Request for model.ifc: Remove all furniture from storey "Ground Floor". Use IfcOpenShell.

First a look at what the model holds.

```python
import ifcopenshell
import ifcopenshell.util.element

model = ifcopenshell.open("model.ifc")
print(model.schema)
storey = next(s for s in model.by_type("IfcBuildingStorey") if s.Name == "Ground Floor")
furniture = [e for e in ifcopenshell.util.element.get_decomposition(storey) if e.is_a("IfcFurnishingElement")]
seen = {}
for e in furniture:
    element_type = ifcopenshell.util.element.get_type(e)
    name = element_type.Name if element_type not in (None, e) else None
    seen[name] = seen.get(name, 0) + 1
for name, count in sorted(seen.items(), key=str):
    print(count, "x", name)
```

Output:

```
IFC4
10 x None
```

```python
import ifcopenshell
import ifcopenshell.api.root
import ifcopenshell.util.element

model = ifcopenshell.open("model.ifc")

storey = next(s for s in model.by_type("IfcBuildingStorey") if s.Name == "Ground Floor")
furniture = [e for e in ifcopenshell.util.element.get_decomposition(storey) if e.is_a("IfcFurnishingElement")]

for e in furniture:
    ifcopenshell.api.root.remove_product(model, product=e)
print(len(furniture), "removed")

model.write("model-out.ifc")
```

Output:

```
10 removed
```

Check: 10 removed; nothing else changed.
